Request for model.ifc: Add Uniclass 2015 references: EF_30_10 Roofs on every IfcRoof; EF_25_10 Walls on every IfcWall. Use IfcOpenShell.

First a look at what the model holds.

```python
import ifcopenshell

model = ifcopenshell.open("model.ifc")
print(model.schema)
print("classifications:", [c.Name for c in model.by_type("IfcClassification")])
for ifc_class in ("IfcDoor", "IfcRoof", "IfcStair", "IfcWall", "IfcWindow"):
    print(ifc_class, len(model.by_type(ifc_class)))
```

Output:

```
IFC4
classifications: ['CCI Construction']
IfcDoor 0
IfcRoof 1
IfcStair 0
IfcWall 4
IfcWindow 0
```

```python
import ifcopenshell
import ifcopenshell.api.classification

model = ifcopenshell.open("model.ifc")

system = ifcopenshell.api.classification.add_classification(model, classification="Uniclass 2015")

codes = {
    "IfcRoof": ("EF_30_10", "Roofs"),
    "IfcWall": ("EF_25_10", "Walls"),
}
for ifc_class, (code, name) in codes.items():
    products = model.by_type(ifc_class)
    ifcopenshell.api.classification.add_reference(
        model, products=products, classification=system, identification=code, name=name
    )
    print(code, len(products))

model.write("model_updated.ifc")
```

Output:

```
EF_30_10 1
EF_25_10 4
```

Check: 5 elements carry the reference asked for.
